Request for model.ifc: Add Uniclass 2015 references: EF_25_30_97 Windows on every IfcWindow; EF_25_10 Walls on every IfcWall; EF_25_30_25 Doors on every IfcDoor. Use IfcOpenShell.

First a look at what the model holds.

```python
import ifcopenshell

model = ifcopenshell.open("model.ifc")
print(model.schema)
print("classifications:", [c.Name for c in model.by_type("IfcClassification")])
for ifc_class in ("IfcDoor", "IfcRoof", "IfcStair", "IfcWall", "IfcWindow"):
    print(ifc_class, len(model.by_type(ifc_class)))
```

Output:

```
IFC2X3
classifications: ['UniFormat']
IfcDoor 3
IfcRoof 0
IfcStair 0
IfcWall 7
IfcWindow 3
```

```python
import ifcopenshell
import ifcopenshell.api.classification

model = ifcopenshell.open("model.ifc")

# IFC2X3 requires Source and Edition and has no link from the project to the system.
system = model.create_entity("IfcClassification", Source="NBS", Edition="2015", Name="Uniclass 2015")

codes = {
    "IfcWindow": ("EF_25_30_97", "Windows"),
    "IfcWall": ("EF_25_10", "Walls"),
    "IfcDoor": ("EF_25_30_25", "Doors"),
}
for ifc_class, (code, name) in codes.items():
    products = model.by_type(ifc_class)
    ifcopenshell.api.classification.add_reference(
        model, products=products, classification=system, identification=code, name=name
    )
    print(code, len(products))

model.write("model_updated.ifc")
```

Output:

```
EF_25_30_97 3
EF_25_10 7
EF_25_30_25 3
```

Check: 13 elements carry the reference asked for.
